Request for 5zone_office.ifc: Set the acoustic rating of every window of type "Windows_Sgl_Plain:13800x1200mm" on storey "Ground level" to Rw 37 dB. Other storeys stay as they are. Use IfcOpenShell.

First a look at what the model holds.

```python
import ifcopenshell
import ifcopenshell.util.element

model = ifcopenshell.open("5zone_office.ifc")
print(model.schema)
storey = next(s for s in model.by_type("IfcBuildingStorey") if s.Name == "Ground level")
windows = [e for e in ifcopenshell.util.element.get_decomposition(storey) if e.is_a("IfcWindow")]
seen = {}
for e in windows:
    element_type = ifcopenshell.util.element.get_type(e)
    key = (element_type.Name if element_type != e and element_type else None, ifcopenshell.util.element.get_pset(e, "Pset_WindowCommon", "AcousticRating"))
    seen[key] = seen.get(key, 0) + 1
for (name, value), count in sorted(seen.items(), key=str):
    print(count, "x", name, "|", value)
```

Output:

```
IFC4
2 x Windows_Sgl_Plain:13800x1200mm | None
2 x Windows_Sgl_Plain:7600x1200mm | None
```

```python
import ifcopenshell
import ifcopenshell.api.pset
import ifcopenshell.util.element

model = ifcopenshell.open("5zone_office.ifc")

storey = next(s for s in model.by_type("IfcBuildingStorey") if s.Name == "Ground level")
windows = [e for e in ifcopenshell.util.element.get_decomposition(storey) if e.is_a("IfcWindow")]

count = 0
for e in windows:
    element_type = ifcopenshell.util.element.get_type(e)
    if element_type in (None, e) or element_type.Name != "Windows_Sgl_Plain:13800x1200mm":
        continue
    # add_pset returns the element's existing set when there is one.
    pset = ifcopenshell.api.pset.add_pset(model, product=e, name="Pset_WindowCommon")
    ifcopenshell.api.pset.edit_pset(model, pset=pset, properties={"AcousticRating": "Rw 37 dB"})
    count += 1

print(count, "windows updated")

model.write("5zone_office_updated.ifc")
```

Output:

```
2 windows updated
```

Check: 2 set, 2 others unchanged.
